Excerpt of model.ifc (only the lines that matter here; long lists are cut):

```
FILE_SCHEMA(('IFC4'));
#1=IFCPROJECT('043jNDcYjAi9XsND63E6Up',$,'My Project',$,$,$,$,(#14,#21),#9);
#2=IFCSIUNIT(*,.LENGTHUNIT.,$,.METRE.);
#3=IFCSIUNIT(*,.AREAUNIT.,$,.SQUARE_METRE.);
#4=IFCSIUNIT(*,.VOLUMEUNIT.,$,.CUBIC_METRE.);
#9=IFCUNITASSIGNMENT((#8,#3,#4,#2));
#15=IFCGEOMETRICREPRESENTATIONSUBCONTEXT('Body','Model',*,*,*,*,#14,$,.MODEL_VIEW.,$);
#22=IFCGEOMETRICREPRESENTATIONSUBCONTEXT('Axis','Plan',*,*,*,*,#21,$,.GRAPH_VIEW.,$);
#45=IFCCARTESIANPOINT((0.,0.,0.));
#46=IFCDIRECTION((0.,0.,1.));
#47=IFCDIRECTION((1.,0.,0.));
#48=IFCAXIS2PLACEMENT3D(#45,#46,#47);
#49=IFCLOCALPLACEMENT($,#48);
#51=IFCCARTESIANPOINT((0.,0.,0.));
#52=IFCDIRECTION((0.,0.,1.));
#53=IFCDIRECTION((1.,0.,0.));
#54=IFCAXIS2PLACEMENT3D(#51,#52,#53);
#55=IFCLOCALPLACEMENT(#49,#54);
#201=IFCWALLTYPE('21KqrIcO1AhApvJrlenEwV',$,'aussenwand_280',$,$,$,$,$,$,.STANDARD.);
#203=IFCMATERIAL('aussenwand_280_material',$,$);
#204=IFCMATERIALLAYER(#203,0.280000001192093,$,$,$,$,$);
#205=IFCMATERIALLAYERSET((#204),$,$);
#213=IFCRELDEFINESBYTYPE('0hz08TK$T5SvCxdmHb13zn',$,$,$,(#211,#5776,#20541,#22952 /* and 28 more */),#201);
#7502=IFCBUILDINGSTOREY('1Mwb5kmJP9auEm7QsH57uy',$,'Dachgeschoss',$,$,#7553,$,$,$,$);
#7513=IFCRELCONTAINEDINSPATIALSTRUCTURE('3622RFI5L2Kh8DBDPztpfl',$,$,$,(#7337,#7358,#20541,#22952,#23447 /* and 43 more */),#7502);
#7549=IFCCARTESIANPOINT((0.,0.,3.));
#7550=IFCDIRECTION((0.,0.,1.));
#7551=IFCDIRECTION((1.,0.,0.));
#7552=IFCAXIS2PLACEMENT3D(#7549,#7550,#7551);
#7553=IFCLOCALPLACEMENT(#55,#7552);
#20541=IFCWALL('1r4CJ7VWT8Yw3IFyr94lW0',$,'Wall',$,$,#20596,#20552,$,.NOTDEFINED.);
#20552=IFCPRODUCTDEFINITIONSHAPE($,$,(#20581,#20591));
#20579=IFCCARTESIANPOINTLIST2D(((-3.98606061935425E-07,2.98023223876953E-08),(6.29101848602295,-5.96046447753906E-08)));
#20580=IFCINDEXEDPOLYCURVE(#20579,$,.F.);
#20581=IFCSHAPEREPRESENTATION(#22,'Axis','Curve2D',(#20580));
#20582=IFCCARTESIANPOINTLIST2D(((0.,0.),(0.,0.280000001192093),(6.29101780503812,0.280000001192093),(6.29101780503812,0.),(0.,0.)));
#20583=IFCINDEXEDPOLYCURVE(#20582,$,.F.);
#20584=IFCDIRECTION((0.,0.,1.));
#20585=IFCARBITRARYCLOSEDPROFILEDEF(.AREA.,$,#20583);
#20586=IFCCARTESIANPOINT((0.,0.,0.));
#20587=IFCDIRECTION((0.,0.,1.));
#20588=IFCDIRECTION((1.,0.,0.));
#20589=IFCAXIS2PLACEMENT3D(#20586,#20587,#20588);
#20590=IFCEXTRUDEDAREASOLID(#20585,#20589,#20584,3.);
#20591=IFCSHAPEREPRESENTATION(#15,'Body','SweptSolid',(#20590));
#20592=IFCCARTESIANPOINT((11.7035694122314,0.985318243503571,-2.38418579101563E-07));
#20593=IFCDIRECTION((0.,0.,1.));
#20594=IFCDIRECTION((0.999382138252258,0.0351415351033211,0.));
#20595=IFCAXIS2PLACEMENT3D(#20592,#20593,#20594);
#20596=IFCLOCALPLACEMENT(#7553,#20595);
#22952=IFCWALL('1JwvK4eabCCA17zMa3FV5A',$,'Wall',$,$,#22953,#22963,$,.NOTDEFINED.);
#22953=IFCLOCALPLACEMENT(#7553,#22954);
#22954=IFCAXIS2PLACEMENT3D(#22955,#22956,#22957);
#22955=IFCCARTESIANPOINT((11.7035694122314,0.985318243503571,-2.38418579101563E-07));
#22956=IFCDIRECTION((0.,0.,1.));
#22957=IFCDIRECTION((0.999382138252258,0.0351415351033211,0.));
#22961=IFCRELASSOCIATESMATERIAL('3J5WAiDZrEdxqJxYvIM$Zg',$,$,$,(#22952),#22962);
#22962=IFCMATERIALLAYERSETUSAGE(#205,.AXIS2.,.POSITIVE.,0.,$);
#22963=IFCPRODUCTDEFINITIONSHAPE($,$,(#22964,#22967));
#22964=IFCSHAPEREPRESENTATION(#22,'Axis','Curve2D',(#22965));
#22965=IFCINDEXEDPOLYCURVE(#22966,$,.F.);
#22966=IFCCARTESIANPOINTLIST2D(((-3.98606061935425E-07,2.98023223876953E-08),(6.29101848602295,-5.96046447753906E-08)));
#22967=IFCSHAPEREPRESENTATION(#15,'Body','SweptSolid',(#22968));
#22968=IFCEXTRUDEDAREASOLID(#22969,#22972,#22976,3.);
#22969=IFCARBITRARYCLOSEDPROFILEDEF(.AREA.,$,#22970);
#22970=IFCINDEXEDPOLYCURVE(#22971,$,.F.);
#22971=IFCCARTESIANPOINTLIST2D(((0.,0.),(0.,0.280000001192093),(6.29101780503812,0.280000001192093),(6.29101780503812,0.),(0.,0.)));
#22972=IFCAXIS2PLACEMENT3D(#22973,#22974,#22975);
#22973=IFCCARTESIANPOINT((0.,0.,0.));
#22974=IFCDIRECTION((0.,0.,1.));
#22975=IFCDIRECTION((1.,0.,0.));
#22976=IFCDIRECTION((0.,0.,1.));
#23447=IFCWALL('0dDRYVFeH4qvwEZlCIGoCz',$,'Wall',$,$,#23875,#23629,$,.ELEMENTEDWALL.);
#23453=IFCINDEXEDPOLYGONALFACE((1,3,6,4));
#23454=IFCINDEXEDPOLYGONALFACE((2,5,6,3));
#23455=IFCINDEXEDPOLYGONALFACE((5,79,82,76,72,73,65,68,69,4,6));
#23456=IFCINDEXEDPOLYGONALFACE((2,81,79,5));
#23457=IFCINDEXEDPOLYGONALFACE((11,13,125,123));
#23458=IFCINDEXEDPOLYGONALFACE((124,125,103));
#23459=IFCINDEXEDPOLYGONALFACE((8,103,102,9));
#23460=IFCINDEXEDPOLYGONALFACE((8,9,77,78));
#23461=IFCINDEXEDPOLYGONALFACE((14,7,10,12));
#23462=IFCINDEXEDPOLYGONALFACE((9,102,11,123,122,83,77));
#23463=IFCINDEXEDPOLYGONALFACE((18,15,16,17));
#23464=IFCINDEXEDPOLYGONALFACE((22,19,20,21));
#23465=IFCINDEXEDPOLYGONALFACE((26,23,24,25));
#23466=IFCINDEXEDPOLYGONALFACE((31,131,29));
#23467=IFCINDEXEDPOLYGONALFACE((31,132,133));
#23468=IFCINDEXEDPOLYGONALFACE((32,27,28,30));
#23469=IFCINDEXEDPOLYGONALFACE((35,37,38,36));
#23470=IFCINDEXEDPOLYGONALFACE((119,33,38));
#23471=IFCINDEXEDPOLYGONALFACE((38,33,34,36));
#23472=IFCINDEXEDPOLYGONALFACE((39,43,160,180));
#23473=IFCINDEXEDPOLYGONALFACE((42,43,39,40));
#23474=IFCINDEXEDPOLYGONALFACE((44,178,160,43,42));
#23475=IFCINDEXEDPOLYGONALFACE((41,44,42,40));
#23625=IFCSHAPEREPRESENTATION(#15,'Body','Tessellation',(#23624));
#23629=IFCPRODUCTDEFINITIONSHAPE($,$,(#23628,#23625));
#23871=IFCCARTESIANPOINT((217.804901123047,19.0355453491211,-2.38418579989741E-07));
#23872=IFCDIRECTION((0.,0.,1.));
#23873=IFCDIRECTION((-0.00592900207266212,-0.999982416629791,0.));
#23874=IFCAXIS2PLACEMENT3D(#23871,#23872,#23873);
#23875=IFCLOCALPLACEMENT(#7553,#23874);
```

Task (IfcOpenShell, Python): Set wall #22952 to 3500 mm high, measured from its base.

```python
import ifcopenshell
import ifcopenshell.geom
import ifcopenshell.util.representation
import ifcopenshell.util.shape
import ifcopenshell.util.unit

model = ifcopenshell.open("model.ifc")
unit_scale = ifcopenshell.util.unit.calculate_unit_scale(model)
settings = ifcopenshell.geom.settings()


def volume(element):
    """Net volume in cubic metres, openings subtracted."""
    shape = ifcopenshell.geom.create_shape(settings, element)
    return ifcopenshell.util.shape.get_volume(shape.geometry)


wall = model.by_guid("1JwvK4eabCCA17zMa3FV5A")
before = volume(wall)

body = ifcopenshell.util.representation.get_representation(wall, "Model", "Body")
solid = body.Items[0]
old_height = solid.Depth
solid.Depth = 3.5 / unit_scale
after = volume(wall)

print(f"height {old_height:g} -> {solid.Depth:g}, volume {before:.3f} -> {after:.3f} m3")

model.write("model_edited.ifc")
```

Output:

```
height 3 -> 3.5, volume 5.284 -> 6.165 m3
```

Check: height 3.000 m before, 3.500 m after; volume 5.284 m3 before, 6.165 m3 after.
